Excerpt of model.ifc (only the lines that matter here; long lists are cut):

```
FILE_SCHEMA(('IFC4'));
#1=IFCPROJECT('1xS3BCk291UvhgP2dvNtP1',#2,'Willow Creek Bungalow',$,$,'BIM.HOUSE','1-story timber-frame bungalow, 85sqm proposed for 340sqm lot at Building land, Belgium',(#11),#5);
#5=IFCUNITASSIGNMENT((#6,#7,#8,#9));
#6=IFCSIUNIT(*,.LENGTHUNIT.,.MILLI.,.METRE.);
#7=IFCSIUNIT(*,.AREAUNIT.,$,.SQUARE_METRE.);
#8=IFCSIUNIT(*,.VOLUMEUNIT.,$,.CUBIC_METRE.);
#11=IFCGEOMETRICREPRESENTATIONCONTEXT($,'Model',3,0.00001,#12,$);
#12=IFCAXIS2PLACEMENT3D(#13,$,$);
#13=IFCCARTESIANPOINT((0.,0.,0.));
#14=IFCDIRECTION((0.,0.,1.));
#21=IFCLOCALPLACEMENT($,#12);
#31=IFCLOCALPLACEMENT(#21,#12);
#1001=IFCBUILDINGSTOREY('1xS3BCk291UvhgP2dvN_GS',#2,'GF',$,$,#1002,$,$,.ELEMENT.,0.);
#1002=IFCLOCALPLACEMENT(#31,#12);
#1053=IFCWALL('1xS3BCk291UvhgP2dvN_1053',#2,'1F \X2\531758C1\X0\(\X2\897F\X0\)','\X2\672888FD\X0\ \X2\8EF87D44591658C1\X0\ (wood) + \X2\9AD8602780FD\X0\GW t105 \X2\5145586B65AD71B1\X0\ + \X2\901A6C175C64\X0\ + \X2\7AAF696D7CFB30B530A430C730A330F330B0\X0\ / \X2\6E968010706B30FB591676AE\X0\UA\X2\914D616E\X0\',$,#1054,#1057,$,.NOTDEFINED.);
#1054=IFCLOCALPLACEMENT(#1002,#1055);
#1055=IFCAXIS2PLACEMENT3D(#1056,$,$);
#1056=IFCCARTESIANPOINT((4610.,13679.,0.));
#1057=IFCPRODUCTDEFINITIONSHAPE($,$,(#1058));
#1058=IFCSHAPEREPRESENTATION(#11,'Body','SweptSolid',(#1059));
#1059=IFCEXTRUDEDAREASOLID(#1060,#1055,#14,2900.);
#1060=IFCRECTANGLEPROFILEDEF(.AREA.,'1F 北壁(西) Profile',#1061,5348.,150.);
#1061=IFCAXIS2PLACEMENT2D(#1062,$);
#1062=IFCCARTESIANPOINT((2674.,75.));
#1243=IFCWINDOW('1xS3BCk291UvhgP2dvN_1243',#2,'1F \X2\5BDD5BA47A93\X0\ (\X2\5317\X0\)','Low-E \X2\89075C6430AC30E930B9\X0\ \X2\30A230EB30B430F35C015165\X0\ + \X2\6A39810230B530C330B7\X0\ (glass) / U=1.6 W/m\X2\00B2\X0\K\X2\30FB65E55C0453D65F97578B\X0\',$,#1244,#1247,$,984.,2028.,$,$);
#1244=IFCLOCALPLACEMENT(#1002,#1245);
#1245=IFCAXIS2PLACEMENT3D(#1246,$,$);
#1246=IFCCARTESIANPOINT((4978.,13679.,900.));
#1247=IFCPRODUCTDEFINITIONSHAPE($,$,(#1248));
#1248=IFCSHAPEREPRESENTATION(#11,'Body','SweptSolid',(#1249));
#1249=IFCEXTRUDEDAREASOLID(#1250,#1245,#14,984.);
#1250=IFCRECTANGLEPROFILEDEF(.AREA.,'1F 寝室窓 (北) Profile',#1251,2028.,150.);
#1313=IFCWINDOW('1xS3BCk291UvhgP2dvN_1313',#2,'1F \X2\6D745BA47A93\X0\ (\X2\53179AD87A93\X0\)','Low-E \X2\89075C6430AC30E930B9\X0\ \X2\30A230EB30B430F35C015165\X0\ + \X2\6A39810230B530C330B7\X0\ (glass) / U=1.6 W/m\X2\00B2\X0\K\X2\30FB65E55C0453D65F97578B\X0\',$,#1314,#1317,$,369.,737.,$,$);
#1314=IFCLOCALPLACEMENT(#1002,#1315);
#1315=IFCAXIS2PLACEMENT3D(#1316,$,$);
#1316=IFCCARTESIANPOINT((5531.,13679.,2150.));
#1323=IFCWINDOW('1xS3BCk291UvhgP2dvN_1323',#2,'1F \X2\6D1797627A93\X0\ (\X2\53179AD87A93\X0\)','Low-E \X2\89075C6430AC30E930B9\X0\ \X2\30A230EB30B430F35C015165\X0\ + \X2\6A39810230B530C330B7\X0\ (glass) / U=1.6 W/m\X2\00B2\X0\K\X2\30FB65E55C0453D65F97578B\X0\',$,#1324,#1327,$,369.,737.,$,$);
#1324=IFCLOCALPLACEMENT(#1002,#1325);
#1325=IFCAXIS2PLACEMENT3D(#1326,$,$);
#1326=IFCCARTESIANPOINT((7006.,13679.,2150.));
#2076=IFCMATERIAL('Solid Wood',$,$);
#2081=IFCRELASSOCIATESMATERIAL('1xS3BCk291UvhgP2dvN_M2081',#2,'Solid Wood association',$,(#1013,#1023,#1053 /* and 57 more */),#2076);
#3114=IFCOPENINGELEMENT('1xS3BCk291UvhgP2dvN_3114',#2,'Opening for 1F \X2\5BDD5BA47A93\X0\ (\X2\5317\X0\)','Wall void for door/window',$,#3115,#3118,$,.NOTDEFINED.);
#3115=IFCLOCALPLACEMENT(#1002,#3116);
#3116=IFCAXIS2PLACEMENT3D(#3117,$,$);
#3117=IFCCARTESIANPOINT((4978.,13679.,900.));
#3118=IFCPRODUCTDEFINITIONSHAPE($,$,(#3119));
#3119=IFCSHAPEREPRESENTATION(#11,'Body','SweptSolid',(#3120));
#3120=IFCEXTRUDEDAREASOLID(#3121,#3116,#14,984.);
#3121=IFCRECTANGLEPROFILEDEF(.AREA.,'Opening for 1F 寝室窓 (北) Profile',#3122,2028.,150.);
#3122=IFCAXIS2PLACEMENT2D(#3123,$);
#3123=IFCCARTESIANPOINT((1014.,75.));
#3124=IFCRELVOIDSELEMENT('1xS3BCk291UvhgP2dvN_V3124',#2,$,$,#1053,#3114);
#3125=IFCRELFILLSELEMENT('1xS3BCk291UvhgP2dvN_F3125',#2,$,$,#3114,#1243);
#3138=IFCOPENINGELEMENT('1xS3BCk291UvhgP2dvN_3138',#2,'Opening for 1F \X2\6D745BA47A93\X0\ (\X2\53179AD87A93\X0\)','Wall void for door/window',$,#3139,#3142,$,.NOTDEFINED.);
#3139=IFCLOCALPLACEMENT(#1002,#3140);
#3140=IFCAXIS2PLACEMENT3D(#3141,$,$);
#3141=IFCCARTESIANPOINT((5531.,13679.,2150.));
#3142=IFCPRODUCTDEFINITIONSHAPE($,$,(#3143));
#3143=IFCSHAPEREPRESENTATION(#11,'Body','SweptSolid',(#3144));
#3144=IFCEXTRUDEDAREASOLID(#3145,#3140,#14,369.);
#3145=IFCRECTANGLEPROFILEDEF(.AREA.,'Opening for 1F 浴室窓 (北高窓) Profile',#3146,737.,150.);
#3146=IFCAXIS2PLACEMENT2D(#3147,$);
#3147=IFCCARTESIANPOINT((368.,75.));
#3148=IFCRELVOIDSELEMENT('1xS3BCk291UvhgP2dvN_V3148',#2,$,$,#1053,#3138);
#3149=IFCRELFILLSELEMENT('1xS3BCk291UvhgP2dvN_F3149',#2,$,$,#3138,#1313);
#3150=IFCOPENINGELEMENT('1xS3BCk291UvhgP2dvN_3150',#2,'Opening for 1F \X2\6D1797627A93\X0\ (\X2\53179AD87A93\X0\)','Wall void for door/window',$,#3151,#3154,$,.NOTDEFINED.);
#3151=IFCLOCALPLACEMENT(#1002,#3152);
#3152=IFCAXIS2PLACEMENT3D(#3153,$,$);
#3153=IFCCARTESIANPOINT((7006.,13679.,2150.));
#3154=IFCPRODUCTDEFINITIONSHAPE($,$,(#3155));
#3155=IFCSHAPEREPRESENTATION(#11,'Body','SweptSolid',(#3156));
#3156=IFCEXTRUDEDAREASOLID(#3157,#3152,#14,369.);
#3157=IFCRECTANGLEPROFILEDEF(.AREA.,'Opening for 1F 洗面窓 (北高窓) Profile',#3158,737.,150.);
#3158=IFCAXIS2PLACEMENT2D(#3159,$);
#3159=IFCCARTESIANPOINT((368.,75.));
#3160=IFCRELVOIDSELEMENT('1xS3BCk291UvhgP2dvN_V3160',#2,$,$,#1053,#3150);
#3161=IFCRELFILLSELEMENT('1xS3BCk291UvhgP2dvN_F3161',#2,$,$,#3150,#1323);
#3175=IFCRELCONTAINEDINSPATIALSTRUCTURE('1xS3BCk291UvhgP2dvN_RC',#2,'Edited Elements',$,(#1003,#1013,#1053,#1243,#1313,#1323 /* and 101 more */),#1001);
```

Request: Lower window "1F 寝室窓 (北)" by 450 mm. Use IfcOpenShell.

```python
import numpy as np
import ifcopenshell
import ifcopenshell.api.geometry
import ifcopenshell.util.placement
import ifcopenshell.util.unit

model = ifcopenshell.open("model.ifc")
unit_scale = ifcopenshell.util.unit.calculate_unit_scale(model)

window = model.by_guid("1xS3BCk291UvhgP2dvN_1243")
opening = window.FillsVoids[0].RelatingOpeningElement
dz = -0.45 / unit_scale

shift = np.array([0.0, 0.0, dz])
# The window is not placed relative to its opening, so move both.
for product in (opening, window):
    matrix = ifcopenshell.util.placement.get_local_placement(product.ObjectPlacement)
    matrix[:3, 3] += shift
    ifcopenshell.api.geometry.edit_object_placement(model, product=product, matrix=matrix, is_si=False)

print(f"moved by {dz * unit_scale:+.3f} m")

model.write("model_updated.ifc")
```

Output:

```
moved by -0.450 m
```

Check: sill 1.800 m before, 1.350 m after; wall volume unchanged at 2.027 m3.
